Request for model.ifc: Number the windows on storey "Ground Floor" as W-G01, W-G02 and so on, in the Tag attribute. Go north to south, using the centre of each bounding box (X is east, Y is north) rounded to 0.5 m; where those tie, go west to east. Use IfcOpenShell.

First a look at what the model holds.

```python
import ifcopenshell
import ifcopenshell.util.element
import ifcopenshell.util.placement

model = ifcopenshell.open("model.ifc")
print(model.schema)
storey = next(s for s in model.by_type("IfcBuildingStorey") if s.Name == "Ground Floor")
windows = [e for e in ifcopenshell.util.element.get_decomposition(storey) if e.is_a("IfcWindow")]
for e in sorted(windows, key=lambda e: e.id()):
    origin = ifcopenshell.util.placement.get_local_placement(e.ObjectPlacement)[:3, 3]
    print(e.id(), e.Tag, e.Name, origin.round(2) + 0.0, sep=" | ")
```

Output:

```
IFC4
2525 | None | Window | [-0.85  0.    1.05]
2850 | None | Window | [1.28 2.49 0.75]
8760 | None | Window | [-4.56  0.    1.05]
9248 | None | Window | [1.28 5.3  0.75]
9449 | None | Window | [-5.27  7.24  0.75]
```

```python
import ifcopenshell
import ifcopenshell.geom
import ifcopenshell.util.element
import ifcopenshell.util.shape

model = ifcopenshell.open("model.ifc")
settings = ifcopenshell.geom.settings()
settings.set("use-world-coords", True)


def centre(element):
    shape = ifcopenshell.geom.create_shape(settings, element)
    return ifcopenshell.util.shape.get_bbox_centroid(shape.geometry)


storey = next(s for s in model.by_type("IfcBuildingStorey") if s.Name == "Ground Floor")
windows = [e for e in ifcopenshell.util.element.get_decomposition(storey) if e.is_a("IfcWindow")]

# Insertion points can sit at a corner or the storey origin, so sort by the geometry (in metres).
centres = {e: centre(e) for e in windows}
windows.sort(key=lambda e: (-round(centres[e][1] / 0.5), centres[e][0]))

for i, e in enumerate(windows, start=1):
    number = f"W-G{i:02d}"
    e.Tag = number
    print(e.id(), number)

model.write("model_v2.ifc")
```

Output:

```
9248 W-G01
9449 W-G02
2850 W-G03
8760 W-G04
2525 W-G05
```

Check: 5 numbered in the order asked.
